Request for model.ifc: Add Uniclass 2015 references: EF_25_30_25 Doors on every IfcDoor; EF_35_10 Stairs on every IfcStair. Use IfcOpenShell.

First a look at what the model holds.

```python
import ifcopenshell

model = ifcopenshell.open("model.ifc")
print(model.schema)
print("classifications:", [c.Name for c in model.by_type("IfcClassification")])
for ifc_class in ("IfcDoor", "IfcRoof", "IfcStair", "IfcWall", "IfcWindow"):
    print(ifc_class, len(model.by_type(ifc_class)))
```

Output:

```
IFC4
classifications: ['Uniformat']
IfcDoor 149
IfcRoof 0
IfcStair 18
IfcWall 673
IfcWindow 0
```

```python
import ifcopenshell
import ifcopenshell.api.classification

model = ifcopenshell.open("model.ifc")

system = ifcopenshell.api.classification.add_classification(model, classification="Uniclass 2015")

codes = {
    "IfcDoor": ("EF_25_30_25", "Doors"),
    "IfcStair": ("EF_35_10", "Stairs"),
}
for ifc_class, (code, name) in codes.items():
    products = model.by_type(ifc_class)
    ifcopenshell.api.classification.add_reference(
        model, products=products, classification=system, identification=code, name=name
    )
    print(code, len(products))

model.write("model_rev.ifc")
```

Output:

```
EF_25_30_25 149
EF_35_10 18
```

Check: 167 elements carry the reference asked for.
